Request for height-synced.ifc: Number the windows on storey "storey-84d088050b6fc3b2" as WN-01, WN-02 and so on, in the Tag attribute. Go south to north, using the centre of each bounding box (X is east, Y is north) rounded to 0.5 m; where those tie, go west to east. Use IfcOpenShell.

First a look at what the model holds.

```python
import ifcopenshell
import ifcopenshell.util.element
import ifcopenshell.util.placement

model = ifcopenshell.open("height-synced.ifc")
print(model.schema)
storey = next(s for s in model.by_type("IfcBuildingStorey") if s.Name == "storey-84d088050b6fc3b2")
windows = [e for e in ifcopenshell.util.element.get_decomposition(storey) if e.is_a("IfcWindow")]
for e in sorted(windows, key=lambda e: e.id()):
    origin = ifcopenshell.util.placement.get_local_placement(e.ObjectPlacement)[:3, 3]
    print(e.id(), e.Tag, e.Name, origin.round(2) + 0.0, sep=" | ")
```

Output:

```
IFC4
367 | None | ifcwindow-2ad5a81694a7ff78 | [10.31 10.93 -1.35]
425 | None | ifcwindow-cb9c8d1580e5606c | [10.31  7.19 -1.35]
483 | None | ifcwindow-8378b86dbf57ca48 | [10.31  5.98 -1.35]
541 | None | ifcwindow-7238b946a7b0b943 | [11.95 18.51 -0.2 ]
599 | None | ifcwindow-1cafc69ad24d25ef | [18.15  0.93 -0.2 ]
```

```python
import ifcopenshell
import ifcopenshell.geom
import ifcopenshell.util.element
import ifcopenshell.util.shape

model = ifcopenshell.open("height-synced.ifc")
settings = ifcopenshell.geom.settings()
settings.set("use-world-coords", True)


def centre(element):
    shape = ifcopenshell.geom.create_shape(settings, element)
    return ifcopenshell.util.shape.get_bbox_centroid(shape.geometry)


storey = next(s for s in model.by_type("IfcBuildingStorey") if s.Name == "storey-84d088050b6fc3b2")
windows = [e for e in ifcopenshell.util.element.get_decomposition(storey) if e.is_a("IfcWindow")]

# Insertion points can sit at a corner or the storey origin, so sort by the geometry (in metres).
centres = {e: centre(e) for e in windows}
windows.sort(key=lambda e: (round(centres[e][1] / 0.5), centres[e][0]))

for i, e in enumerate(windows, start=1):
    number = f"WN-{i:02d}"
    e.Tag = number
    print(e.id(), number)

model.write("height-synced_v2.ifc")
```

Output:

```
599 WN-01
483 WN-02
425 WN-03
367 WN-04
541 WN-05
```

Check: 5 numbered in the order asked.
